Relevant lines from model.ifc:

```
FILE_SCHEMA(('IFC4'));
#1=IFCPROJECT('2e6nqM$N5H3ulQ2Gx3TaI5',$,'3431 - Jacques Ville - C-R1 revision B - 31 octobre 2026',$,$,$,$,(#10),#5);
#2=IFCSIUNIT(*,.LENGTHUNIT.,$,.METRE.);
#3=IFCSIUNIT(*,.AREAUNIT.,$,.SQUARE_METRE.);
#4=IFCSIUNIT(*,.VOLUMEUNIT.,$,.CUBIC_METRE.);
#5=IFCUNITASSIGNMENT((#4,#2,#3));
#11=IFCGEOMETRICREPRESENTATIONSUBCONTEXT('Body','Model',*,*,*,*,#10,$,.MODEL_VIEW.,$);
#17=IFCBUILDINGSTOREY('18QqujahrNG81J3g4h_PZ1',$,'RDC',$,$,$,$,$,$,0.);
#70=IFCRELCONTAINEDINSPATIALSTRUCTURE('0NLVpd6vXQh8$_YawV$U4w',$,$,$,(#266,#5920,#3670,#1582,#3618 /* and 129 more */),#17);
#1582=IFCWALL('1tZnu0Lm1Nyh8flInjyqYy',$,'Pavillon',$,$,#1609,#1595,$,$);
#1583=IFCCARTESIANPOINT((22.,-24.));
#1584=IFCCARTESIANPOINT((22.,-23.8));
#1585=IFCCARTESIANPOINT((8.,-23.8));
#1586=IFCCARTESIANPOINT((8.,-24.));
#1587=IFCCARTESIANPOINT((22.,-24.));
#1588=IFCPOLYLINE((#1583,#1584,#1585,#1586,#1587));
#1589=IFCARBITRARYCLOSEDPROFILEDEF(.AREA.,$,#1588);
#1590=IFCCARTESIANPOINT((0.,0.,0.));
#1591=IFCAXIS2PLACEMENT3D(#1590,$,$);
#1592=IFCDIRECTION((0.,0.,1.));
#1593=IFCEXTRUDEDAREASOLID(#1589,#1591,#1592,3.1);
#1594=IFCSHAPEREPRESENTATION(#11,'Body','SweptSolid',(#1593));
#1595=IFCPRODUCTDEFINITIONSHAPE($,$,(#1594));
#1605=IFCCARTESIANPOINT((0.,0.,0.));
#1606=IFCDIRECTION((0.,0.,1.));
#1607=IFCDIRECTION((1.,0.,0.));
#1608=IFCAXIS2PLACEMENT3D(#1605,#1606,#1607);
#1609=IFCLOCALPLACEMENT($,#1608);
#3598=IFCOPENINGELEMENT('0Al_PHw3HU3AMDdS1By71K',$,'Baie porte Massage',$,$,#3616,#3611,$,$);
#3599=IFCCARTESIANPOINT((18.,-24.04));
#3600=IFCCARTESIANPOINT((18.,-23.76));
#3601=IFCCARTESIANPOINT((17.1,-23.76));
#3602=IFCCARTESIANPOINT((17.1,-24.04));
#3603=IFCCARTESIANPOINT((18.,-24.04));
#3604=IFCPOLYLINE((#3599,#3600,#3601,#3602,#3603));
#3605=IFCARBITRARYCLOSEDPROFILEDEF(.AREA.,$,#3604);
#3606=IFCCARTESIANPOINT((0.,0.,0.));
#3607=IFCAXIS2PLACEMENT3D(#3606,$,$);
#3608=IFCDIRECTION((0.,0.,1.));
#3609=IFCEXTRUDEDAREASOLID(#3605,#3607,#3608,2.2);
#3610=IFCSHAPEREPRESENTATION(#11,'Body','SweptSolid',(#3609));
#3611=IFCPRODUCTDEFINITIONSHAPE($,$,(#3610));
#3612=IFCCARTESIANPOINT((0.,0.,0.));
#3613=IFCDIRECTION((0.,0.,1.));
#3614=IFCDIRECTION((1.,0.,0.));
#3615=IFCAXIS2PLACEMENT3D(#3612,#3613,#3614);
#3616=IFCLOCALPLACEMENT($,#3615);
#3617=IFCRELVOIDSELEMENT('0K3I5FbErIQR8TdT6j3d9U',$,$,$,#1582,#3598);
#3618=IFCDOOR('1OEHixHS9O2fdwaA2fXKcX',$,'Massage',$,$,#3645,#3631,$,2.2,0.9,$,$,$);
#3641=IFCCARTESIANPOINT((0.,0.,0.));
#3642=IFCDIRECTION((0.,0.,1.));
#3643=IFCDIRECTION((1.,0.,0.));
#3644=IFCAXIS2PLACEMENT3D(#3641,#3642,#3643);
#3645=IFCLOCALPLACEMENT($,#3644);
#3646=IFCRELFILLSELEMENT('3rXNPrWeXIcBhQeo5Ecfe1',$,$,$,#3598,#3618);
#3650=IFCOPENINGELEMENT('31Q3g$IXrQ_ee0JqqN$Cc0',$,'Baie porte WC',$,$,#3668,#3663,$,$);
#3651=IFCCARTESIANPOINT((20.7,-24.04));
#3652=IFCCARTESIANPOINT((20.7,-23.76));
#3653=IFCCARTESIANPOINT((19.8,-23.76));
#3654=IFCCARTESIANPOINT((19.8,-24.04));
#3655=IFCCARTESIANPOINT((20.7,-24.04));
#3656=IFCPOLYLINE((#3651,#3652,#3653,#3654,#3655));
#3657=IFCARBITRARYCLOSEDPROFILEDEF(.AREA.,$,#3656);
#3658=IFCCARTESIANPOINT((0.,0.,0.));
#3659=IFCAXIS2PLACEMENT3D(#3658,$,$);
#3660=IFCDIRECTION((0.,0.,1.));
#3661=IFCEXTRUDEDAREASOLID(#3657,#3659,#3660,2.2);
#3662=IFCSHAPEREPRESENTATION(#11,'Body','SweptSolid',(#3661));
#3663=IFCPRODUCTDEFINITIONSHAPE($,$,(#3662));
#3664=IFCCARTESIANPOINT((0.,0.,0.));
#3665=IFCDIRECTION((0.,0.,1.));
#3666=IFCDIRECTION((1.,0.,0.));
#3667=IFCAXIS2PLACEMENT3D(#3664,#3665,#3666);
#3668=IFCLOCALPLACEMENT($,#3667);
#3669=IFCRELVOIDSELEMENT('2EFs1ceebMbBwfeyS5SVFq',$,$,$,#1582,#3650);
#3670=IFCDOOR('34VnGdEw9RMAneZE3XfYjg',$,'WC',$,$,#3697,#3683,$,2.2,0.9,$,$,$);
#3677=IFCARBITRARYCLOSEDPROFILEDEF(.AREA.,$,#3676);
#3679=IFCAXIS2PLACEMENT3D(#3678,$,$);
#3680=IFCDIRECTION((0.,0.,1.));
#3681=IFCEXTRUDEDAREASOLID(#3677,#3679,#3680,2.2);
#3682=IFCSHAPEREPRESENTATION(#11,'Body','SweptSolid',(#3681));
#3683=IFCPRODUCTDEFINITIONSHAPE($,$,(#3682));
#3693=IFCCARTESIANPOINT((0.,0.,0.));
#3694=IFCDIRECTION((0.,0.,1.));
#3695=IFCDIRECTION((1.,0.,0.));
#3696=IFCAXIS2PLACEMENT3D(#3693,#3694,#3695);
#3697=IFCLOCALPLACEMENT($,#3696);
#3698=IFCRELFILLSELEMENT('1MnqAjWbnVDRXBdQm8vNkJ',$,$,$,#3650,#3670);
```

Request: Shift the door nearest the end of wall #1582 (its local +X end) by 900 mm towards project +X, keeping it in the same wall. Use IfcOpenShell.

```python
import ifcopenshell
import ifcopenshell.api.geometry
import ifcopenshell.util.placement
import ifcopenshell.util.unit

model = ifcopenshell.open("model.ifc")
unit_scale = ifcopenshell.util.unit.calculate_unit_scale(model)

door = model.by_guid("34VnGdEw9RMAneZE3XfYjg")
opening = door.FillsVoids[0].RelatingOpeningElement
wall = opening.VoidsElements[0].RelatingBuildingElement

wall_matrix = ifcopenshell.util.placement.get_local_placement(wall.ObjectPlacement)
shift = wall_matrix[:3, 0] * 0.9 / unit_scale
before = ifcopenshell.util.placement.get_local_placement(door.ObjectPlacement)[:3, 3].copy()

# The door is not placed relative to its opening, so move both.
for product in (opening, door):
    matrix = ifcopenshell.util.placement.get_local_placement(product.ObjectPlacement)
    matrix[:3, 3] += shift
    ifcopenshell.api.geometry.edit_object_placement(model, product=product, matrix=matrix, is_si=False)

after = ifcopenshell.util.placement.get_local_placement(door.ObjectPlacement)[:3, 3]
print("door moved by", (after - before).round(3) + 0.0)

model.write("model_rev.ifc")
```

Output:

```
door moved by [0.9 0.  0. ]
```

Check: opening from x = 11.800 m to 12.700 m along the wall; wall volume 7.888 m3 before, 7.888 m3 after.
